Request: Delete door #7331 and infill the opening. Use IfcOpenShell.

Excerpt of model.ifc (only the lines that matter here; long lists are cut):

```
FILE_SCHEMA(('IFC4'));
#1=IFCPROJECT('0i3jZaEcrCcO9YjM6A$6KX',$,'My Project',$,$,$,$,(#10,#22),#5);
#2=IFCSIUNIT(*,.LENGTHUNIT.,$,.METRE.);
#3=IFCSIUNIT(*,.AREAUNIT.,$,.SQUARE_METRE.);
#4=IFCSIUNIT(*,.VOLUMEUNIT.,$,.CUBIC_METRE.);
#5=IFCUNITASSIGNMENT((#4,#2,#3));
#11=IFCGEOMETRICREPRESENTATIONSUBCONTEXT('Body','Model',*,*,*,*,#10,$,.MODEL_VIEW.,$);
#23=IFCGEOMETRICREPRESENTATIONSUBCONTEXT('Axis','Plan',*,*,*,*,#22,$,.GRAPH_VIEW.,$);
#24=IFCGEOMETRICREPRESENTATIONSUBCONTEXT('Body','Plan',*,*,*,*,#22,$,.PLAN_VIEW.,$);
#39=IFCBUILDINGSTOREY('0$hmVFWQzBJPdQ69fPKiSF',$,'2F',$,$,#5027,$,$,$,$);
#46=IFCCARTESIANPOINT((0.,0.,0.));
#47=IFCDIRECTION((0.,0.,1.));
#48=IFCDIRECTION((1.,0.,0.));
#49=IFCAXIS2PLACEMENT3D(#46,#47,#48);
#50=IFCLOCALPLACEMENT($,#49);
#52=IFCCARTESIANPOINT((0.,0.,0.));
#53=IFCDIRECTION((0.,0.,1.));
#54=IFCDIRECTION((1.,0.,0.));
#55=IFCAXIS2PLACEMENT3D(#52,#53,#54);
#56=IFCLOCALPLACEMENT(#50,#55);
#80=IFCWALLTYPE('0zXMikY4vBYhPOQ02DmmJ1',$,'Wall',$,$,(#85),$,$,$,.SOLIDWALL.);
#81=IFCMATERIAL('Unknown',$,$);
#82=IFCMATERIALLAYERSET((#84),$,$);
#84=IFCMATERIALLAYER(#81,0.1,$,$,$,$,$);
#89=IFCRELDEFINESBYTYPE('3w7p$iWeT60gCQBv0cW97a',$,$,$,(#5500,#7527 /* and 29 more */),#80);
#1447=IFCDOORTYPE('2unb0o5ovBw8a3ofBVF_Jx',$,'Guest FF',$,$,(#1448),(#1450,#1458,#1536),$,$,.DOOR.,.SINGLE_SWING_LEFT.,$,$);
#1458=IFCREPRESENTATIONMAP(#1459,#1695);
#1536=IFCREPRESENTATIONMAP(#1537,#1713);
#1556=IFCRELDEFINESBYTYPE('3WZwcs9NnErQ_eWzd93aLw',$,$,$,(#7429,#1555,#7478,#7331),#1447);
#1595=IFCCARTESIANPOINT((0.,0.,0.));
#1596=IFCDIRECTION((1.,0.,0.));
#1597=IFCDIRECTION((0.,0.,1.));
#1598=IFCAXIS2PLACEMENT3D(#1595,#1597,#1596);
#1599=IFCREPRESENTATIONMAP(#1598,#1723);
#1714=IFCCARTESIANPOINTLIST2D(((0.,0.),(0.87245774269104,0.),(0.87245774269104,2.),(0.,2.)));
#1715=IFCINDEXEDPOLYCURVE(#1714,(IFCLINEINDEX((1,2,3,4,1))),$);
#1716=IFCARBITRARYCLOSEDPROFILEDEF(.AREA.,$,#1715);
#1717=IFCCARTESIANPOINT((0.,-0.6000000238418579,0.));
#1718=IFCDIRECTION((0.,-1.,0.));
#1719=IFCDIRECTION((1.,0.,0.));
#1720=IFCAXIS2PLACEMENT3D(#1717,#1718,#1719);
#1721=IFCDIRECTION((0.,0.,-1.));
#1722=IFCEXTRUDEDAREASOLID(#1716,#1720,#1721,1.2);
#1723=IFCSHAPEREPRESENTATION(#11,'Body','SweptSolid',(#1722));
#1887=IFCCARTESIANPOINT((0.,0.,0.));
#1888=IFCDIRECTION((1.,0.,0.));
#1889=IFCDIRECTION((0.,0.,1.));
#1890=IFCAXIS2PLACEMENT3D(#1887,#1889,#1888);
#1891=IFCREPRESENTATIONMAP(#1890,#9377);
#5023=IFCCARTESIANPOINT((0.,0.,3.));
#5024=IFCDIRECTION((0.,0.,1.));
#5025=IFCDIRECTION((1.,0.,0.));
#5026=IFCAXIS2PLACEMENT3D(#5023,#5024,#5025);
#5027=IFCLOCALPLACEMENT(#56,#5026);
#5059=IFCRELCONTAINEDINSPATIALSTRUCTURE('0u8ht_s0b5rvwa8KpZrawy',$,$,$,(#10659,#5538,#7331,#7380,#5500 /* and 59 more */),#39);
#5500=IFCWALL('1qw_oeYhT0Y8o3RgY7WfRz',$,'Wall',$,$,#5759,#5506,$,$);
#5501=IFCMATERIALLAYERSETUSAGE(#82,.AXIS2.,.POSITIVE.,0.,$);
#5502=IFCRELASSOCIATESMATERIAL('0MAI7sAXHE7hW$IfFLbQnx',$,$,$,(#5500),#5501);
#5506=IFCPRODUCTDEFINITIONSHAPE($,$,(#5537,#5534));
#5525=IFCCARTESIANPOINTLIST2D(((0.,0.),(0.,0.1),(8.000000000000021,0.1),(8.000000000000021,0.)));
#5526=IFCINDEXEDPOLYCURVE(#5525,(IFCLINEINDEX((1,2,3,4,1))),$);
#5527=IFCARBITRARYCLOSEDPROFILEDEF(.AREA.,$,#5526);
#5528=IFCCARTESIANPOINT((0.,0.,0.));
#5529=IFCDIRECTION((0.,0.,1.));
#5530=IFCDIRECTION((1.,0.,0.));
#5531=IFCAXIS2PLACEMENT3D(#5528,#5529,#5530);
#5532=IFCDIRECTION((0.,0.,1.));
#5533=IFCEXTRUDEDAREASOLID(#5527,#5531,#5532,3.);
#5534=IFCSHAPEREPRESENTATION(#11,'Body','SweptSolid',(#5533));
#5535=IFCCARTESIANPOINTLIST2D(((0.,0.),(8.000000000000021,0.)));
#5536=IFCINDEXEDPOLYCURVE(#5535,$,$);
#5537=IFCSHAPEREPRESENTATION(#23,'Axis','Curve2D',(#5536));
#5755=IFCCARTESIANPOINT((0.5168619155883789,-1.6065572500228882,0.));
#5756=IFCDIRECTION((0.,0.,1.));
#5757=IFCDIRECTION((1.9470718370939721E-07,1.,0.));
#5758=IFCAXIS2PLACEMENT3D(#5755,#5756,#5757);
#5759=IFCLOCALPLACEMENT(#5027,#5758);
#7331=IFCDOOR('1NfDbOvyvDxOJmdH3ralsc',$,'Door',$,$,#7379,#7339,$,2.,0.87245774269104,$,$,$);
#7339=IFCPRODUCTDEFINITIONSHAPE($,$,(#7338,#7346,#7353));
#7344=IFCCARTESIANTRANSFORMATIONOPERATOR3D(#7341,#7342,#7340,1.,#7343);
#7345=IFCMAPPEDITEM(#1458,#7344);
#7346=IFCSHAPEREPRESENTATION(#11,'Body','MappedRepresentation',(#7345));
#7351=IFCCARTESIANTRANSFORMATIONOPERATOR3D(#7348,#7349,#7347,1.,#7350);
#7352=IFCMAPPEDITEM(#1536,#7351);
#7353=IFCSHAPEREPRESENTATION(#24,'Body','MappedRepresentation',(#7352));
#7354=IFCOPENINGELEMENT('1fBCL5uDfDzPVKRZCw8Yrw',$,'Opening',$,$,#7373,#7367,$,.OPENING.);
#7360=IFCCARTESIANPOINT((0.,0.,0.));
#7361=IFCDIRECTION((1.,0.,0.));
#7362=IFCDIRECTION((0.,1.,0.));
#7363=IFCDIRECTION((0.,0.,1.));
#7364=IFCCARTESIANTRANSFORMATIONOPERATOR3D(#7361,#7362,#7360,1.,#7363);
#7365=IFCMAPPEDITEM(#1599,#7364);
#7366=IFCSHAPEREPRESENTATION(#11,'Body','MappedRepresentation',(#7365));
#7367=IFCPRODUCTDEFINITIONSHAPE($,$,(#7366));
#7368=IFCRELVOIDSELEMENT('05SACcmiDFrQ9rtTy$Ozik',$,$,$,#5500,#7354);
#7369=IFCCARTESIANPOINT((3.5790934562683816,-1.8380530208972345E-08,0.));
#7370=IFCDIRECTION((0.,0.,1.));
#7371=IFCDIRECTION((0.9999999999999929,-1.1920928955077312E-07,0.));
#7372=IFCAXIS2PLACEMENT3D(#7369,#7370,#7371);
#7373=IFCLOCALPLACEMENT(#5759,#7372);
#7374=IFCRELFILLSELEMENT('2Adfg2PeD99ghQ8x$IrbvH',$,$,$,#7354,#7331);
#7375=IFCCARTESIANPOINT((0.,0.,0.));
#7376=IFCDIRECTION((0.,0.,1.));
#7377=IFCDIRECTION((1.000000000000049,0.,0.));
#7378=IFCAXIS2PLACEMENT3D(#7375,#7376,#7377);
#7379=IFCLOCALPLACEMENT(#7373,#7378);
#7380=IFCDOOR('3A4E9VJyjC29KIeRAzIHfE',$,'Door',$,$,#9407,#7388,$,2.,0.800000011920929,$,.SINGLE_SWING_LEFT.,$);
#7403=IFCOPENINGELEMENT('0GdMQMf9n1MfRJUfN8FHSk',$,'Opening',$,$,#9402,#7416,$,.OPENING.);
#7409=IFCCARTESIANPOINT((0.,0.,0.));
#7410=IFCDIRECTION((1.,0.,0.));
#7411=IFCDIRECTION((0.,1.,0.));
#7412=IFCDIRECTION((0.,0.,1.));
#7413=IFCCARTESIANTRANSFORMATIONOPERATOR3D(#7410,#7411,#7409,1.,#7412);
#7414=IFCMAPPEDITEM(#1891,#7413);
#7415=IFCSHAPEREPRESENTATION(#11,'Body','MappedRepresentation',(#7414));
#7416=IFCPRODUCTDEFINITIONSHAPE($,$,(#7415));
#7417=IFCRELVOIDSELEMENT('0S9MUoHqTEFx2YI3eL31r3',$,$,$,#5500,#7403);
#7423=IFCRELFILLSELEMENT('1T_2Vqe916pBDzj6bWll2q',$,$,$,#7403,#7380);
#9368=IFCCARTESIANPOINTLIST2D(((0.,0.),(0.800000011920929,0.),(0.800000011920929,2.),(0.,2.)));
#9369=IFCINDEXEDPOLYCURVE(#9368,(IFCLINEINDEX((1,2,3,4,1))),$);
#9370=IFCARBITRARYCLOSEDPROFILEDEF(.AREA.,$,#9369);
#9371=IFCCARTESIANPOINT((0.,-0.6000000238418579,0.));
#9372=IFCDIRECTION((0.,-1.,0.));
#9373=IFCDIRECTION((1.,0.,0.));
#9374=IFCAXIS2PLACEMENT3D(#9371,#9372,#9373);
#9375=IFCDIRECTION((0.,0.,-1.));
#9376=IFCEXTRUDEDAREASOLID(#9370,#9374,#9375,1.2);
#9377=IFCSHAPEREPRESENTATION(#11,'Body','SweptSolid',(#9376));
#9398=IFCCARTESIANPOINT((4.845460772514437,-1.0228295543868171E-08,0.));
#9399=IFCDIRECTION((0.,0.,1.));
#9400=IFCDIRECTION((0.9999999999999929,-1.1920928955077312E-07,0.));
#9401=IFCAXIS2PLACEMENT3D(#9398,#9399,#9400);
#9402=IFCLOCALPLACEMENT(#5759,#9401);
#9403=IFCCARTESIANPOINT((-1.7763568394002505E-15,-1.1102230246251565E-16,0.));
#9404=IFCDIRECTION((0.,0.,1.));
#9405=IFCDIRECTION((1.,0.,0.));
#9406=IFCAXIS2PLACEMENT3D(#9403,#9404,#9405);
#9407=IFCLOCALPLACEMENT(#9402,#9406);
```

```python
import ifcopenshell
import ifcopenshell.api.feature
import ifcopenshell.api.root
import ifcopenshell.geom
import ifcopenshell.util.shape

model = ifcopenshell.open("model.ifc")
settings = ifcopenshell.geom.settings()


def volume(element):
    """Net volume in cubic metres, openings subtracted."""
    shape = ifcopenshell.geom.create_shape(settings, element)
    return ifcopenshell.util.shape.get_volume(shape.geometry)


door = model.by_guid("1NfDbOvyvDxOJmdH3ralsc")
opening = door.FillsVoids[0].RelatingOpeningElement
wall = opening.VoidsElements[0].RelatingBuildingElement
before = volume(wall)

ifcopenshell.api.root.remove_product(model, product=door)
ifcopenshell.api.feature.remove_feature(model, feature=opening)

after = volume(wall)

print(f"wall volume {before:.3f} -> {after:.3f} m3")

model.write("model-out.ifc")
```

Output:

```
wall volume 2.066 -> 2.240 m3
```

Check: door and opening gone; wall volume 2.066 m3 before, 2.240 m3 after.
